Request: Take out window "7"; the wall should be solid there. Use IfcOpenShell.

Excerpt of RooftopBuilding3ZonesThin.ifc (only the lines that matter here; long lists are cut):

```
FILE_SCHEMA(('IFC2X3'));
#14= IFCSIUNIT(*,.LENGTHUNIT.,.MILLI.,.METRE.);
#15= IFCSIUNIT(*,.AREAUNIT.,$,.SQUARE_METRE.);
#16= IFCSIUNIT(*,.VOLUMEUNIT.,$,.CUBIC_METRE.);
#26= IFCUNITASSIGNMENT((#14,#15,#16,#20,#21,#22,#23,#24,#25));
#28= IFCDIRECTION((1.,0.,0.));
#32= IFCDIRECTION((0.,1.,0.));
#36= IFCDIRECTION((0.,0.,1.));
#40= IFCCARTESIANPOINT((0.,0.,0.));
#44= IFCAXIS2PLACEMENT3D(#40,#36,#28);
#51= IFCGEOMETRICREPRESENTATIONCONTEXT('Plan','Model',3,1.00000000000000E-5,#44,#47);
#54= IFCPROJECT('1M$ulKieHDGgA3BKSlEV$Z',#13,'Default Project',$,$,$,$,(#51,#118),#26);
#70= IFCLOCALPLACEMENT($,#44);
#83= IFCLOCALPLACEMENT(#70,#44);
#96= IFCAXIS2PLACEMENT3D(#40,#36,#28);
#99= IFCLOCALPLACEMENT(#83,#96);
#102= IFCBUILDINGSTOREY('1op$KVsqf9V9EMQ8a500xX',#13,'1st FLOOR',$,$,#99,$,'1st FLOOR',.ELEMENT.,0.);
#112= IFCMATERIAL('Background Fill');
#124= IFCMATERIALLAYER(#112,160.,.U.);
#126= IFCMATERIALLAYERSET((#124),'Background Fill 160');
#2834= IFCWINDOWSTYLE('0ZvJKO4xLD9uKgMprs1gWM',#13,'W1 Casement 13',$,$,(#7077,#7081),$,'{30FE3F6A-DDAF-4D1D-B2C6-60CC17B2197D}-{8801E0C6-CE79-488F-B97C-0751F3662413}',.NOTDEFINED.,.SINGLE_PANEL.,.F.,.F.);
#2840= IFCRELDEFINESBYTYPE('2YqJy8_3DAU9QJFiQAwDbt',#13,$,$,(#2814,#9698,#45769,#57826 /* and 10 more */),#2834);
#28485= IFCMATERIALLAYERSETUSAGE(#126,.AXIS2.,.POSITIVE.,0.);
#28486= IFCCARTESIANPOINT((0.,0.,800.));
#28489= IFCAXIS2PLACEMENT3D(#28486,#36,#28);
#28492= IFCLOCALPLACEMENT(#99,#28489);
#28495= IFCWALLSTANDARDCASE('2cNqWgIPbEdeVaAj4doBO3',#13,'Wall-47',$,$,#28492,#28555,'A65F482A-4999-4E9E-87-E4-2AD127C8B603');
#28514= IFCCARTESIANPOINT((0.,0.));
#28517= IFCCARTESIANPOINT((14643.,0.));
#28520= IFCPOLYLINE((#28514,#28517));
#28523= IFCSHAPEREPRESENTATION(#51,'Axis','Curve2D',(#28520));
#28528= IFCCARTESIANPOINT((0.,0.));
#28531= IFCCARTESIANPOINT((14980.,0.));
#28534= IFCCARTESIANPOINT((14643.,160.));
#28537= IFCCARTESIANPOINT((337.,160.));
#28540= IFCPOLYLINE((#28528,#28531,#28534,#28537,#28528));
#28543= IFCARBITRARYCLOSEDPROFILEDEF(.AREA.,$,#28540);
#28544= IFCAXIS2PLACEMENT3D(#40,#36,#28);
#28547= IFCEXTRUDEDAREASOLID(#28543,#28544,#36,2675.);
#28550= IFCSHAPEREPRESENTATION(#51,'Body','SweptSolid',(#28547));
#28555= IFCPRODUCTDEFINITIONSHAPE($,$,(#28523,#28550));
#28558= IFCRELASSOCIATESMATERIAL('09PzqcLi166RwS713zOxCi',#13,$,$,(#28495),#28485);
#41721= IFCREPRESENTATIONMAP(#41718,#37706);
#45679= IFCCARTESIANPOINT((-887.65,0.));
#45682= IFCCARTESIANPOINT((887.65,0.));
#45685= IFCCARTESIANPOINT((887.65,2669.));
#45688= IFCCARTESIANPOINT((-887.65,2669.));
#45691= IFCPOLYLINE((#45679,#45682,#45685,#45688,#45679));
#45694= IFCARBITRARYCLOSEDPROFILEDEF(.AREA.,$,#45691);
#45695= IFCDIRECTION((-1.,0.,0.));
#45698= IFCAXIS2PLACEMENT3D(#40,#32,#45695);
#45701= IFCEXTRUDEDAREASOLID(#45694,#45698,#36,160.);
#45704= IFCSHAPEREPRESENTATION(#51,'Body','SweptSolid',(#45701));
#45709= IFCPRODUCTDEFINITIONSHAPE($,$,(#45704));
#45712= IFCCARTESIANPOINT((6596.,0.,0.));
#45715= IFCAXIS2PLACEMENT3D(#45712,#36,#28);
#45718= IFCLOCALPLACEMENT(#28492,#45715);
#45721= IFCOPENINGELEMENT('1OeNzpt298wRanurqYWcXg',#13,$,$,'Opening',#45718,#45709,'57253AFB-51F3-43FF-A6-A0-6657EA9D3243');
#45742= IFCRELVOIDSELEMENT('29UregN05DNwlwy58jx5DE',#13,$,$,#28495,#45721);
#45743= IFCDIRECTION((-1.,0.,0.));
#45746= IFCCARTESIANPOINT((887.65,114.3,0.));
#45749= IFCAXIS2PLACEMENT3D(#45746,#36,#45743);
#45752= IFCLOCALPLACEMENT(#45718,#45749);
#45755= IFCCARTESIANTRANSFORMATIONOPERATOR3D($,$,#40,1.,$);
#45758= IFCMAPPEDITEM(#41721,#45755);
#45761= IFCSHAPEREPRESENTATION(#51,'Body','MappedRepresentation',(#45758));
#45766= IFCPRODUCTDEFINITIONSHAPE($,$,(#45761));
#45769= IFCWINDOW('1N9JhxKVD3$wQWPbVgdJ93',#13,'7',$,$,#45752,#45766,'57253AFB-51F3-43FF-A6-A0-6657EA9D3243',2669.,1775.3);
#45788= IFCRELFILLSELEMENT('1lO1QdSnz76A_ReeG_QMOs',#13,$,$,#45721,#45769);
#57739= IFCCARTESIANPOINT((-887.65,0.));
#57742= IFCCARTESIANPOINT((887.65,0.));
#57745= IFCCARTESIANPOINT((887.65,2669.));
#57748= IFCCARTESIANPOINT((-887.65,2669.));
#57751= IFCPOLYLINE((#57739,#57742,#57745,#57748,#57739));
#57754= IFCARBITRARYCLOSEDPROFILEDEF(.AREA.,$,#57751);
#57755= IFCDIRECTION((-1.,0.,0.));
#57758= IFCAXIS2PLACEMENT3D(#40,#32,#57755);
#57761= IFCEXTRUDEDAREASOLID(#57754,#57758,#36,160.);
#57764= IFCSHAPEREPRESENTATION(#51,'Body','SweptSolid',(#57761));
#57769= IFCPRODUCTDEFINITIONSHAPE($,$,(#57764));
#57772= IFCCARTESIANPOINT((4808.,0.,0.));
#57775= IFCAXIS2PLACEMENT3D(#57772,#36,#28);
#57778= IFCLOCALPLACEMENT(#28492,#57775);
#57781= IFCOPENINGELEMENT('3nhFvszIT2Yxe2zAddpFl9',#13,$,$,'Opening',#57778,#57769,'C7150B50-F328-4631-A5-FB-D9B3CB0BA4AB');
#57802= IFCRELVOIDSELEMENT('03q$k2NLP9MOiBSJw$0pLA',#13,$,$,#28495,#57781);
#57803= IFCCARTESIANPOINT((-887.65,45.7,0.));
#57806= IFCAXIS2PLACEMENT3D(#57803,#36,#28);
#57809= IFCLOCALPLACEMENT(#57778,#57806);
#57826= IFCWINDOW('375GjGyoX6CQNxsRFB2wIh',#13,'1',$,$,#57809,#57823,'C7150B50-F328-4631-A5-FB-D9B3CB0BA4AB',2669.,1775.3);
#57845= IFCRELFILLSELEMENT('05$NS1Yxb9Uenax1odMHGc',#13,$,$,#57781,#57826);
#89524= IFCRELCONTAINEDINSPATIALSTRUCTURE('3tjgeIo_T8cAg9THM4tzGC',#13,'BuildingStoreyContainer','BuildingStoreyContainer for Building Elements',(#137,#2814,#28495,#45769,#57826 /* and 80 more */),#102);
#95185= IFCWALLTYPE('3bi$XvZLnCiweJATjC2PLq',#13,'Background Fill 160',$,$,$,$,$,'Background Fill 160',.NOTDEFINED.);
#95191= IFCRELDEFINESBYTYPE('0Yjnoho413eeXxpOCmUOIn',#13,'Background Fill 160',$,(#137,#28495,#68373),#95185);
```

```python
import ifcopenshell
import ifcopenshell.api.feature
import ifcopenshell.api.root
import ifcopenshell.geom
import ifcopenshell.util.shape

model = ifcopenshell.open("RooftopBuilding3ZonesThin.ifc")
settings = ifcopenshell.geom.settings()


def volume(element):
    """Net volume in cubic metres, openings subtracted."""
    shape = ifcopenshell.geom.create_shape(settings, element)
    return ifcopenshell.util.shape.get_volume(shape.geometry)


window = model.by_id(45769)
opening = window.FillsVoids[0].RelatingOpeningElement
wall = opening.VoidsElements[0].RelatingBuildingElement
before = volume(wall)

ifcopenshell.api.root.remove_product(model, product=window)
ifcopenshell.api.feature.remove_feature(model, feature=opening)

after = volume(wall)

print(f"wall volume {before:.3f} -> {after:.3f} m3")

model.write("RooftopBuilding3ZonesThin-out.ifc")
```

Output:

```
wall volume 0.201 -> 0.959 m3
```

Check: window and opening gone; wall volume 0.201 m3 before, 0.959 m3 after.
